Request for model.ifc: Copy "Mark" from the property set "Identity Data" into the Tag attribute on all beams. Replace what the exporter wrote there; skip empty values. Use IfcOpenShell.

First a look at what the model holds.

```python
import ifcopenshell
import ifcopenshell.util.element

model = ifcopenshell.open("model.ifc")
print(model.schema)
beams = model.by_type("IfcBeam")
print(len(beams), "beams")
for e in beams[:8]:
    source = ifcopenshell.util.element.get_pset(e, "Identity Data", "Mark")
    target = e.Tag
    print(e.id(), repr(source), repr(target), sep=" | ")
```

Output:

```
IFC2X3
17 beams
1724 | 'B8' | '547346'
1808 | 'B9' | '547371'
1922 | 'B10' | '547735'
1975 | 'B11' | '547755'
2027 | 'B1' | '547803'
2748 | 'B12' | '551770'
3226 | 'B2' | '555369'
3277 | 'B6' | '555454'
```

```python
import ifcopenshell
import ifcopenshell.util.element

model = ifcopenshell.open("model.ifc")

count = 0
for e in model.by_type("IfcBeam"):
    value = ifcopenshell.util.element.get_pset(e, "Identity Data", "Mark")
    current = e.Tag
    if not value or not value.strip() or current == value:
        continue
    e.Tag = value
    count += 1

print(count, "beams updated")

model.write("model_v2.ifc")
```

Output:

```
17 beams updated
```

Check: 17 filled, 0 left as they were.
